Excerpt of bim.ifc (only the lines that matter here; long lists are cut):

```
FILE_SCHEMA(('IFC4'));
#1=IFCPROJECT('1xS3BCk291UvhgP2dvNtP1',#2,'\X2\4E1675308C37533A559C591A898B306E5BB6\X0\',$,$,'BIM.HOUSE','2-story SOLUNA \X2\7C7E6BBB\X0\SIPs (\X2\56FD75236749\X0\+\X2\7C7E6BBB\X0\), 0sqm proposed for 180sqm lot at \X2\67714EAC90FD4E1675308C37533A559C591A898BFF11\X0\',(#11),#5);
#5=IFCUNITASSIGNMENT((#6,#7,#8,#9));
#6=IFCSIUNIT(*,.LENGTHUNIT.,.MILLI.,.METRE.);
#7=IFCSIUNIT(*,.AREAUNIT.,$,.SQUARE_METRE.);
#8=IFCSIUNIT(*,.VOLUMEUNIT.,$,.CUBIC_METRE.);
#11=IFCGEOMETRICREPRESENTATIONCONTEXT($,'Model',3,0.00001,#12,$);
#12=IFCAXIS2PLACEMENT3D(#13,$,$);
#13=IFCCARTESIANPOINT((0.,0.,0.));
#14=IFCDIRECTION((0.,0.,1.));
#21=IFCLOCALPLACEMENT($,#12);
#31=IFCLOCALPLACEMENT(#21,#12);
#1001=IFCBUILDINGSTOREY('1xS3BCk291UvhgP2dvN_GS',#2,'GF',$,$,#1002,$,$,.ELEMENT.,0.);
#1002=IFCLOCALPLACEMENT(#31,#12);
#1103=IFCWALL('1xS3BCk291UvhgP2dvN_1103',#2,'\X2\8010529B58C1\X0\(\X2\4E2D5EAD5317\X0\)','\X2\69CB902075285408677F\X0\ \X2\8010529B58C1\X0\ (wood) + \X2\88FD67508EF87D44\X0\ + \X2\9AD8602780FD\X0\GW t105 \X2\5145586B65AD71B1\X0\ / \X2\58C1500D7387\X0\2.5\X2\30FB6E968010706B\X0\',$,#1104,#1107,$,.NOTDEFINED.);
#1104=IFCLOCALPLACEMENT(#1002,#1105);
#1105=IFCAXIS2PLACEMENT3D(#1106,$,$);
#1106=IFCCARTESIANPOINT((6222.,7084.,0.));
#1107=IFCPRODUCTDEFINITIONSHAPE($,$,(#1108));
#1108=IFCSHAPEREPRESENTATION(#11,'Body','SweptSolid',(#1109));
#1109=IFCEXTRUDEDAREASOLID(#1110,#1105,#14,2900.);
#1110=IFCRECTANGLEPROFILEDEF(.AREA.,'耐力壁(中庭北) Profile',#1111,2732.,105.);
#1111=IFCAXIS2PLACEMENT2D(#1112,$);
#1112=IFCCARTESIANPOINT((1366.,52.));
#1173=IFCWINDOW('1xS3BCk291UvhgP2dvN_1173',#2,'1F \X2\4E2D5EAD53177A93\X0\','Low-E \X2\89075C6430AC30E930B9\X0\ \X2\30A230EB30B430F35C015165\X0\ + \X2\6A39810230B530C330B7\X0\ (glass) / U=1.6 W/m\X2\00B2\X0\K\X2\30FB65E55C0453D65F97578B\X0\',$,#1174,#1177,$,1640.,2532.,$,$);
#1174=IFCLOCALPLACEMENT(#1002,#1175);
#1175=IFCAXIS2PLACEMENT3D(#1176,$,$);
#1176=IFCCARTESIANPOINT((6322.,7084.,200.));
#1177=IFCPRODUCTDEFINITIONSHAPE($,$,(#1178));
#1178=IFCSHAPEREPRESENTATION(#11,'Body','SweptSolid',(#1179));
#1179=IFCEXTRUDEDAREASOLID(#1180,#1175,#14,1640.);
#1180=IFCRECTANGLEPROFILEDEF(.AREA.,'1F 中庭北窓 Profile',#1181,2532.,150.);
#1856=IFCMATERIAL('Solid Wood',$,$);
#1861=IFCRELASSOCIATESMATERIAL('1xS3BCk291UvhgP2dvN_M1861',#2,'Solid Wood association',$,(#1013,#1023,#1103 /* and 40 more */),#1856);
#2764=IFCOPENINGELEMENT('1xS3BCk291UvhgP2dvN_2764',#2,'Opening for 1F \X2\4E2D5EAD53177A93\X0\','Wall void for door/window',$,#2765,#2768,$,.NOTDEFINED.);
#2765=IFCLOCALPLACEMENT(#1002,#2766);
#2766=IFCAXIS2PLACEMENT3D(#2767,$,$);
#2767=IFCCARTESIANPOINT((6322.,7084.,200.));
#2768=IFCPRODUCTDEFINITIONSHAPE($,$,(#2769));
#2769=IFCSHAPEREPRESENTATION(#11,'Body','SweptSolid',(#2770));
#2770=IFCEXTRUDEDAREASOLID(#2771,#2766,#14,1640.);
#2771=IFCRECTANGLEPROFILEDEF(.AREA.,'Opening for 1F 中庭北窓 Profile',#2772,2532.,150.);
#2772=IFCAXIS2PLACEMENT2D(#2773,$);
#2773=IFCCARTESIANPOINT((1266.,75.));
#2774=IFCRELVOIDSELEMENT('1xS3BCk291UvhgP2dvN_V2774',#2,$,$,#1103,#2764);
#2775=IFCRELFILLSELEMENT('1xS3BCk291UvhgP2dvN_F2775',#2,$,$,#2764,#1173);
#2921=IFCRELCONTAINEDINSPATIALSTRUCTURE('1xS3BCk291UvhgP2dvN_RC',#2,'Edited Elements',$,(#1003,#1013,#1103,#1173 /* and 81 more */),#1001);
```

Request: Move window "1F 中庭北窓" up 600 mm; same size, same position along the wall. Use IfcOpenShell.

```python
import numpy as np
import ifcopenshell
import ifcopenshell.api.geometry
import ifcopenshell.util.placement
import ifcopenshell.util.unit

model = ifcopenshell.open("bim.ifc")
unit_scale = ifcopenshell.util.unit.calculate_unit_scale(model)

window = model.by_guid("1xS3BCk291UvhgP2dvN_1173")
opening = window.FillsVoids[0].RelatingOpeningElement
dz = 600.0

shift = np.array([0.0, 0.0, dz])
# The window is not placed relative to its opening, so move both.
for product in (opening, window):
    matrix = ifcopenshell.util.placement.get_local_placement(product.ObjectPlacement)
    matrix[:3, 3] += shift
    ifcopenshell.api.geometry.edit_object_placement(model, product=product, matrix=matrix, is_si=False)

print(f"moved by {dz * unit_scale:+.3f} m")

model.write("bim_edited.ifc")
```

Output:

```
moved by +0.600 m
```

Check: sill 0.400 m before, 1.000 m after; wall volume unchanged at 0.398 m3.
